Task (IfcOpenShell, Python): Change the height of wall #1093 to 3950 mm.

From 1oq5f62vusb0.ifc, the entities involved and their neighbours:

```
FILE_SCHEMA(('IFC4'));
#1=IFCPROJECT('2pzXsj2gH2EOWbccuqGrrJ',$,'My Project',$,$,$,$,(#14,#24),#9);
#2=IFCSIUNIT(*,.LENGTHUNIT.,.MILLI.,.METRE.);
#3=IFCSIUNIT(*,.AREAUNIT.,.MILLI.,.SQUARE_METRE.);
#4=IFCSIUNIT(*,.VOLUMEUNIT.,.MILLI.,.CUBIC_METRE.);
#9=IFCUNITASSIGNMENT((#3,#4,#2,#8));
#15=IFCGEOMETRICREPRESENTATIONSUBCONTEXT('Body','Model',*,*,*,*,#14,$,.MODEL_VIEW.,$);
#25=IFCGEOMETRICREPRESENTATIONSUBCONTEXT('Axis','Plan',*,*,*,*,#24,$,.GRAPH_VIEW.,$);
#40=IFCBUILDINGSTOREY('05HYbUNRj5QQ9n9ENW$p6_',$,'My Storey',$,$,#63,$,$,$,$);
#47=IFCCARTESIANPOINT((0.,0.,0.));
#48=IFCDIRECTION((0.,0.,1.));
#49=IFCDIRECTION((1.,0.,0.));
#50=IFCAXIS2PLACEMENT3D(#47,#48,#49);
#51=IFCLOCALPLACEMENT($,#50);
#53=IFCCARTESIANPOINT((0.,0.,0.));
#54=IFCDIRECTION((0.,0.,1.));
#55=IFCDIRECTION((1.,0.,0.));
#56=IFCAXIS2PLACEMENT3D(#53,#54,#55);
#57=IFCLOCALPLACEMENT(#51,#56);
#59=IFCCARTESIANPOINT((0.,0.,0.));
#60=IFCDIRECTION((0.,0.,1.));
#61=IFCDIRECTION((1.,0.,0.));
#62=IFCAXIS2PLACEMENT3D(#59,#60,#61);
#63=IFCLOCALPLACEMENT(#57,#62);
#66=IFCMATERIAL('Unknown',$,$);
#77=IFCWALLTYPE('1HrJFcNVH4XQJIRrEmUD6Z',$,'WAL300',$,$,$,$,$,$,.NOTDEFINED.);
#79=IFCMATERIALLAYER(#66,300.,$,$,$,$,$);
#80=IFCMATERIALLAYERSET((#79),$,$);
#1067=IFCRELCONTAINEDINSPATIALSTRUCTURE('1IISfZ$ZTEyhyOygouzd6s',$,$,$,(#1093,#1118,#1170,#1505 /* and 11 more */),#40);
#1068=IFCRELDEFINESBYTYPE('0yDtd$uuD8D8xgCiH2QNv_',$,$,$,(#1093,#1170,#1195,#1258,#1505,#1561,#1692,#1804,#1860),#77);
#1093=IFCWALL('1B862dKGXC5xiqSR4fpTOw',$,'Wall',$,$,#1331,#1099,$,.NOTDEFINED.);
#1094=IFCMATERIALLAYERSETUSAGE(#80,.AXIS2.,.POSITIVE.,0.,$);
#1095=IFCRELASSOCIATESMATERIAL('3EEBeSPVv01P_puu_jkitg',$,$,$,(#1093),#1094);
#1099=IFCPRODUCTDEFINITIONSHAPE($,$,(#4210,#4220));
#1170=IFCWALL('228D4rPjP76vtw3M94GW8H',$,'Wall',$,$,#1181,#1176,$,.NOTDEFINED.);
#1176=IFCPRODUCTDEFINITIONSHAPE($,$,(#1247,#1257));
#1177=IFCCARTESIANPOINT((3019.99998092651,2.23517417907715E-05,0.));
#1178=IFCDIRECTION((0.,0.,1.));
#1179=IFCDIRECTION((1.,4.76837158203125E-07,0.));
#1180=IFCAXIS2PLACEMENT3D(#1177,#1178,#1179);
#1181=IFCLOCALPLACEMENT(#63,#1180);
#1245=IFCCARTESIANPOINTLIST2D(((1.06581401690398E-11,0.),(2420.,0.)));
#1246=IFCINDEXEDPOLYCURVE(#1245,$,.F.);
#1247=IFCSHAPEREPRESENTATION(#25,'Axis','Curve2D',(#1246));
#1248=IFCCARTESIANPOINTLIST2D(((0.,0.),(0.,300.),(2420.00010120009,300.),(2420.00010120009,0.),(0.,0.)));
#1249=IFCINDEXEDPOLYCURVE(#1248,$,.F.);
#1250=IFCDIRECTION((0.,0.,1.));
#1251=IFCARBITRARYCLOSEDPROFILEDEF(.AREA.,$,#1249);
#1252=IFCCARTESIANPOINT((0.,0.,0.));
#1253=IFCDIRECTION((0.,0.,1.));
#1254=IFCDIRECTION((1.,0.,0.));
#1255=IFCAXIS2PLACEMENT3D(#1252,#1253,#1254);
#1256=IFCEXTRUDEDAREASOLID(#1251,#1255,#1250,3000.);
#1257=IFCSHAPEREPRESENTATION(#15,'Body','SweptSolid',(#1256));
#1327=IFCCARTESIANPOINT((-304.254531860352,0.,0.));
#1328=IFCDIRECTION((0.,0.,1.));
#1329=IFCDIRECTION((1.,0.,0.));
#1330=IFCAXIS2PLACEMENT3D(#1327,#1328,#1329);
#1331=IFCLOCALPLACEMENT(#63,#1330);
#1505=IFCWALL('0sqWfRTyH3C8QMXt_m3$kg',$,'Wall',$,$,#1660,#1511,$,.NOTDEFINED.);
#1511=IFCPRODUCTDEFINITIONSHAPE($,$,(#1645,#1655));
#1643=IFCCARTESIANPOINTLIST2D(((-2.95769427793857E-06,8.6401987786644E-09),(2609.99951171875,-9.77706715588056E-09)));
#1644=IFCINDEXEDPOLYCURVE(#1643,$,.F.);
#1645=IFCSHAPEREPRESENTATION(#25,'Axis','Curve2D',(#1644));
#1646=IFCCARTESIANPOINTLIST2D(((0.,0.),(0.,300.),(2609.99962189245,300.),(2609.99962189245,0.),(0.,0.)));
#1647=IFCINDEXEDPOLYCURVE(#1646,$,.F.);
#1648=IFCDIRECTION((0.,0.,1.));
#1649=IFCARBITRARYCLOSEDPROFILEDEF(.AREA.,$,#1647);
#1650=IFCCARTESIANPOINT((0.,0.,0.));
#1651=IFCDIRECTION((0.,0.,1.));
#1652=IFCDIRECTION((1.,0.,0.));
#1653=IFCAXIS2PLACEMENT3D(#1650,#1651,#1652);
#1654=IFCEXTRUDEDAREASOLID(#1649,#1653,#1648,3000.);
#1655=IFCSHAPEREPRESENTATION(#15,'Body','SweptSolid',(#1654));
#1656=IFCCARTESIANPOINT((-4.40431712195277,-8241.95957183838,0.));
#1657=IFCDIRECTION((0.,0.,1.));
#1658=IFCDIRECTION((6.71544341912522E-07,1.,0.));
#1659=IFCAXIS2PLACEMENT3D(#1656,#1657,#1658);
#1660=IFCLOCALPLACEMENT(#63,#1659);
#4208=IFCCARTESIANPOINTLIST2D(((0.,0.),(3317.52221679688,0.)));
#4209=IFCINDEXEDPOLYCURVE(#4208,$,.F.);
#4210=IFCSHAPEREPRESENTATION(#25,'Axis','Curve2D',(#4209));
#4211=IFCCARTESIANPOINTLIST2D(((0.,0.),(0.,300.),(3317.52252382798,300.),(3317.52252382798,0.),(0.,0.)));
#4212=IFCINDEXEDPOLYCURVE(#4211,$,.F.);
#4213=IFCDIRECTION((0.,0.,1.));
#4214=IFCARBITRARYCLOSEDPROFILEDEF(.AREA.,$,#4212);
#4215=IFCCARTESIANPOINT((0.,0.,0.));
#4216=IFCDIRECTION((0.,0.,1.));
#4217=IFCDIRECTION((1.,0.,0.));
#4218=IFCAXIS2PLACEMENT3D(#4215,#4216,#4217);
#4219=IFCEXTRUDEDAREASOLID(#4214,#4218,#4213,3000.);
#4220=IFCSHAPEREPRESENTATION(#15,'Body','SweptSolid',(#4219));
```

```python
import ifcopenshell
import ifcopenshell.geom
import ifcopenshell.util.representation
import ifcopenshell.util.shape

model = ifcopenshell.open("1oq5f62vusb0.ifc")
settings = ifcopenshell.geom.settings()


def volume(element):
    """Net volume in cubic metres, openings subtracted."""
    shape = ifcopenshell.geom.create_shape(settings, element)
    return ifcopenshell.util.shape.get_volume(shape.geometry)


wall = model.by_guid("1B862dKGXC5xiqSR4fpTOw")
before = volume(wall)

body = ifcopenshell.util.representation.get_representation(wall, "Model", "Body")
solid = body.Items[0]
old_height = solid.Depth
solid.Depth = 3950.0
after = volume(wall)

print(f"height {old_height:g} -> {solid.Depth:g}, volume {before:.3f} -> {after:.3f} m3")

model.write("1oq5f62vusb0-out.ifc")
```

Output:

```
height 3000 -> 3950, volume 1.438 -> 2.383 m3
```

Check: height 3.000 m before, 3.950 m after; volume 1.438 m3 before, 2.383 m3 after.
